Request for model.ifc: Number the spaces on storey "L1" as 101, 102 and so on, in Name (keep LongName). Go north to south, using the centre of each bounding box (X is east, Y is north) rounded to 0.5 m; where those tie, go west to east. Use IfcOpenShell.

First a look at what the model holds.

```python
import ifcopenshell
import ifcopenshell.util.element
import ifcopenshell.util.placement

model = ifcopenshell.open("model.ifc")
print(model.schema)
storey = next(s for s in model.by_type("IfcBuildingStorey") if s.Name == "L1")
spaces = [e for e in ifcopenshell.util.element.get_decomposition(storey) if e.is_a("IfcSpace")]
for e in sorted(spaces, key=lambda e: e.id()):
    origin = ifcopenshell.util.placement.get_local_placement(e.ObjectPlacement)[:3, 3]
    print(e.id(), e.Name, e.LongName, origin.round(2) + 0.0, sep=" | ")
```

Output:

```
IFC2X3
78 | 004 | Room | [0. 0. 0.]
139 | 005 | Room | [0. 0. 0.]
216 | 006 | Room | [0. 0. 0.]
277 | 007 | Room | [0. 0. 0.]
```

```python
import ifcopenshell
import ifcopenshell.geom
import ifcopenshell.util.element
import ifcopenshell.util.shape

model = ifcopenshell.open("model.ifc")
settings = ifcopenshell.geom.settings()
settings.set("use-world-coords", True)


def centre(element):
    shape = ifcopenshell.geom.create_shape(settings, element)
    return ifcopenshell.util.shape.get_bbox_centroid(shape.geometry)


storey = next(s for s in model.by_type("IfcBuildingStorey") if s.Name == "L1")
spaces = [e for e in ifcopenshell.util.element.get_decomposition(storey) if e.is_a("IfcSpace")]

# Insertion points can sit at a corner or the storey origin, so sort by the geometry (in metres).
centres = {e: centre(e) for e in spaces}
spaces.sort(key=lambda e: (-round(centres[e][1] / 0.5), centres[e][0]))

for i, e in enumerate(spaces, start=1):
    number = f"1{i:02d}"
    e.Name = number
    print(e.id(), number)

model.write("model-out.ifc")
```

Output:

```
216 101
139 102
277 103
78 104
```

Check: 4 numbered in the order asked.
